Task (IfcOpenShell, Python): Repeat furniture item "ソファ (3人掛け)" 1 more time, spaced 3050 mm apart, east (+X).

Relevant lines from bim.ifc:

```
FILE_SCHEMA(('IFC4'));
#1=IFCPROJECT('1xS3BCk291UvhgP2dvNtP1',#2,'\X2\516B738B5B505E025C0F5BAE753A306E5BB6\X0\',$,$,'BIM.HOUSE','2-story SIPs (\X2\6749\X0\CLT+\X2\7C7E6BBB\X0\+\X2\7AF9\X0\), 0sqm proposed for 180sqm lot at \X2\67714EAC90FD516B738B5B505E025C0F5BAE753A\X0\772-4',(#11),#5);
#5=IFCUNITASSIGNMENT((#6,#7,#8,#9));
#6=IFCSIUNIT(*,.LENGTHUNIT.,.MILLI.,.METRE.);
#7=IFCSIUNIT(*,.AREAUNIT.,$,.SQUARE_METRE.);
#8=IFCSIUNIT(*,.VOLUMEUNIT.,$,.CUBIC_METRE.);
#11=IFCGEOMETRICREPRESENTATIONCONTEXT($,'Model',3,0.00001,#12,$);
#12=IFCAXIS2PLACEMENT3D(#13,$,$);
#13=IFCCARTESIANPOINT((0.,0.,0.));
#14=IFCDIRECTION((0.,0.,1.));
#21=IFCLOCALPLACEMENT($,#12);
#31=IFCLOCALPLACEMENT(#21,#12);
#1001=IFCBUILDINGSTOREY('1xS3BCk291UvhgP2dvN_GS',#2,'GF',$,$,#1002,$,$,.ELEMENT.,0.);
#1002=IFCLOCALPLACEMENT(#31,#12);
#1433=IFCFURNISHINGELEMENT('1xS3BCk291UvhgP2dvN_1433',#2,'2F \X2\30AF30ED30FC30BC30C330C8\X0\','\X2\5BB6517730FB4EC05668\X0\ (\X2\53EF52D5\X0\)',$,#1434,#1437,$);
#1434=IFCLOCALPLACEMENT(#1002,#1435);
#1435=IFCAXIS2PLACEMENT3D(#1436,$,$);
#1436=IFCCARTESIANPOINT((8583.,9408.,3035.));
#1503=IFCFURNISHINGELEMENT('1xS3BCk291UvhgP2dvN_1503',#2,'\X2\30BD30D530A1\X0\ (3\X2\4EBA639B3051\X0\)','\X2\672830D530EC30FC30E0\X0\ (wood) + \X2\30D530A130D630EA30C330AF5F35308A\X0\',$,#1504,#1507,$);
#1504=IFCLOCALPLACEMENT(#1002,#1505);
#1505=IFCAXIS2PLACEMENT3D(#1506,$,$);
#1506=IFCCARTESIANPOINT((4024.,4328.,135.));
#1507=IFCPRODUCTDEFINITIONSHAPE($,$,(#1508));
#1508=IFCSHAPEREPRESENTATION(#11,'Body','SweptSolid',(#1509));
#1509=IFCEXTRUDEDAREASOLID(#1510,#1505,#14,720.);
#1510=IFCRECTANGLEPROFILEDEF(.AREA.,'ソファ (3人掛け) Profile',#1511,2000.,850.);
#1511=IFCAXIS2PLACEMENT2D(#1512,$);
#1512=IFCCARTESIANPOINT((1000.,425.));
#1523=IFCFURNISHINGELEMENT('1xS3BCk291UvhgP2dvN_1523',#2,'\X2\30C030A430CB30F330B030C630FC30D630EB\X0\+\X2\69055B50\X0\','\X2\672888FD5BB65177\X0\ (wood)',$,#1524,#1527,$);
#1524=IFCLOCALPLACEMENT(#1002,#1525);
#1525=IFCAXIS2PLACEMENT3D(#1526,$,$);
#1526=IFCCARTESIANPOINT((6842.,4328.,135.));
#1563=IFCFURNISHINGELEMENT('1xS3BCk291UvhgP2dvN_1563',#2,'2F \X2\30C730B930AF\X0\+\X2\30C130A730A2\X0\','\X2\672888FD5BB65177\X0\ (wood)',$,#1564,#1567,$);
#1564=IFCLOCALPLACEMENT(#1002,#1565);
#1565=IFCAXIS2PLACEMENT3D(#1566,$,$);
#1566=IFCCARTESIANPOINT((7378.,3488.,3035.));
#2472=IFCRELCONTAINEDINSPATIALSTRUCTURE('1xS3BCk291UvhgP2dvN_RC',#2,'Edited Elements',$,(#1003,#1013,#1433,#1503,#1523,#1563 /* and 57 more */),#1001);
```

```python
import numpy as np
import ifcopenshell
import ifcopenshell.api.geometry
import ifcopenshell.api.root
import ifcopenshell.util.element
import ifcopenshell.util.placement

model = ifcopenshell.open("bim.ifc")


def reuse_history(source, copy):
    """copy_class also copies each property set's owner history, people and application; keep the originals."""
    for rel in copy.IsDefinedBy:
        if rel.is_a("IfcRelDefinesByProperties") and (history := rel.RelatingPropertyDefinition.OwnerHistory):
            rel.RelatingPropertyDefinition.OwnerHistory = source.OwnerHistory
            ifcopenshell.util.element.remove_deep2(model, history)


source = model.by_id(1503)
base = ifcopenshell.util.placement.get_local_placement(source.ObjectPlacement)
step = np.array([1.0, 0.0, 0.0]) * 3050.0

for i in range(1, 2):
    copy = ifcopenshell.api.root.copy_class(model, product=source)
    copy.Representation = ifcopenshell.util.element.copy_deep(
        model, source.Representation, exclude=["IfcGeometricRepresentationContext", "IfcRepresentationMap"]
    )
    reuse_history(source, copy)
    matrix = base.copy()
    matrix[:3, 3] += i * step
    print("added at", matrix[:3, 3].round(3) + 0.0)
    ifcopenshell.api.geometry.edit_object_placement(model, product=copy, matrix=matrix, is_si=False)

model.write("bim-out.ifc")
```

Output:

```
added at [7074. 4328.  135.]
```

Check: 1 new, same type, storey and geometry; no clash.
